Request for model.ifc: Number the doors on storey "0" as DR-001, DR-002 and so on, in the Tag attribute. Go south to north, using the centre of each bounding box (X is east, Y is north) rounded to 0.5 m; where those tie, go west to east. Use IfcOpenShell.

First a look at what the model holds.

```python
import ifcopenshell
import ifcopenshell.util.element
import ifcopenshell.util.placement

model = ifcopenshell.open("model.ifc")
print(model.schema)
storey = next(s for s in model.by_type("IfcBuildingStorey") if s.Name == "0")
doors = [e for e in ifcopenshell.util.element.get_decomposition(storey) if e.is_a("IfcDoor")]
for e in sorted(doors, key=lambda e: e.id()):
    origin = ifcopenshell.util.placement.get_local_placement(e.ObjectPlacement)[:3, 3]
    print(e.id(), e.Tag, e.Name, origin.round(2) + 0.0, sep=" | ")
```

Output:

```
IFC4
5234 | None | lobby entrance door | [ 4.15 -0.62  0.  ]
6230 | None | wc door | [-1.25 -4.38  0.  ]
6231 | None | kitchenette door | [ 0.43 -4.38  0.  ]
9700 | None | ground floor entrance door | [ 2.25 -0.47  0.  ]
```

```python
import ifcopenshell
import ifcopenshell.geom
import ifcopenshell.util.element
import ifcopenshell.util.shape

model = ifcopenshell.open("model.ifc")
settings = ifcopenshell.geom.settings()
settings.set("use-world-coords", True)


def centre(element):
    shape = ifcopenshell.geom.create_shape(settings, element)
    return ifcopenshell.util.shape.get_bbox_centroid(shape.geometry)


storey = next(s for s in model.by_type("IfcBuildingStorey") if s.Name == "0")
doors = [e for e in ifcopenshell.util.element.get_decomposition(storey) if e.is_a("IfcDoor")]

# Insertion points can sit at a corner or the storey origin, so sort by the geometry (in metres).
centres = {e: centre(e) for e in doors}
doors.sort(key=lambda e: (round(centres[e][1] / 0.5), centres[e][0]))

for i, e in enumerate(doors, start=1):
    number = f"DR-0{i:02d}"
    e.Tag = number
    print(e.id(), number)

model.write("model-out.ifc")
```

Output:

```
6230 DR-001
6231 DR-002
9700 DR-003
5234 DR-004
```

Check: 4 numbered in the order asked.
